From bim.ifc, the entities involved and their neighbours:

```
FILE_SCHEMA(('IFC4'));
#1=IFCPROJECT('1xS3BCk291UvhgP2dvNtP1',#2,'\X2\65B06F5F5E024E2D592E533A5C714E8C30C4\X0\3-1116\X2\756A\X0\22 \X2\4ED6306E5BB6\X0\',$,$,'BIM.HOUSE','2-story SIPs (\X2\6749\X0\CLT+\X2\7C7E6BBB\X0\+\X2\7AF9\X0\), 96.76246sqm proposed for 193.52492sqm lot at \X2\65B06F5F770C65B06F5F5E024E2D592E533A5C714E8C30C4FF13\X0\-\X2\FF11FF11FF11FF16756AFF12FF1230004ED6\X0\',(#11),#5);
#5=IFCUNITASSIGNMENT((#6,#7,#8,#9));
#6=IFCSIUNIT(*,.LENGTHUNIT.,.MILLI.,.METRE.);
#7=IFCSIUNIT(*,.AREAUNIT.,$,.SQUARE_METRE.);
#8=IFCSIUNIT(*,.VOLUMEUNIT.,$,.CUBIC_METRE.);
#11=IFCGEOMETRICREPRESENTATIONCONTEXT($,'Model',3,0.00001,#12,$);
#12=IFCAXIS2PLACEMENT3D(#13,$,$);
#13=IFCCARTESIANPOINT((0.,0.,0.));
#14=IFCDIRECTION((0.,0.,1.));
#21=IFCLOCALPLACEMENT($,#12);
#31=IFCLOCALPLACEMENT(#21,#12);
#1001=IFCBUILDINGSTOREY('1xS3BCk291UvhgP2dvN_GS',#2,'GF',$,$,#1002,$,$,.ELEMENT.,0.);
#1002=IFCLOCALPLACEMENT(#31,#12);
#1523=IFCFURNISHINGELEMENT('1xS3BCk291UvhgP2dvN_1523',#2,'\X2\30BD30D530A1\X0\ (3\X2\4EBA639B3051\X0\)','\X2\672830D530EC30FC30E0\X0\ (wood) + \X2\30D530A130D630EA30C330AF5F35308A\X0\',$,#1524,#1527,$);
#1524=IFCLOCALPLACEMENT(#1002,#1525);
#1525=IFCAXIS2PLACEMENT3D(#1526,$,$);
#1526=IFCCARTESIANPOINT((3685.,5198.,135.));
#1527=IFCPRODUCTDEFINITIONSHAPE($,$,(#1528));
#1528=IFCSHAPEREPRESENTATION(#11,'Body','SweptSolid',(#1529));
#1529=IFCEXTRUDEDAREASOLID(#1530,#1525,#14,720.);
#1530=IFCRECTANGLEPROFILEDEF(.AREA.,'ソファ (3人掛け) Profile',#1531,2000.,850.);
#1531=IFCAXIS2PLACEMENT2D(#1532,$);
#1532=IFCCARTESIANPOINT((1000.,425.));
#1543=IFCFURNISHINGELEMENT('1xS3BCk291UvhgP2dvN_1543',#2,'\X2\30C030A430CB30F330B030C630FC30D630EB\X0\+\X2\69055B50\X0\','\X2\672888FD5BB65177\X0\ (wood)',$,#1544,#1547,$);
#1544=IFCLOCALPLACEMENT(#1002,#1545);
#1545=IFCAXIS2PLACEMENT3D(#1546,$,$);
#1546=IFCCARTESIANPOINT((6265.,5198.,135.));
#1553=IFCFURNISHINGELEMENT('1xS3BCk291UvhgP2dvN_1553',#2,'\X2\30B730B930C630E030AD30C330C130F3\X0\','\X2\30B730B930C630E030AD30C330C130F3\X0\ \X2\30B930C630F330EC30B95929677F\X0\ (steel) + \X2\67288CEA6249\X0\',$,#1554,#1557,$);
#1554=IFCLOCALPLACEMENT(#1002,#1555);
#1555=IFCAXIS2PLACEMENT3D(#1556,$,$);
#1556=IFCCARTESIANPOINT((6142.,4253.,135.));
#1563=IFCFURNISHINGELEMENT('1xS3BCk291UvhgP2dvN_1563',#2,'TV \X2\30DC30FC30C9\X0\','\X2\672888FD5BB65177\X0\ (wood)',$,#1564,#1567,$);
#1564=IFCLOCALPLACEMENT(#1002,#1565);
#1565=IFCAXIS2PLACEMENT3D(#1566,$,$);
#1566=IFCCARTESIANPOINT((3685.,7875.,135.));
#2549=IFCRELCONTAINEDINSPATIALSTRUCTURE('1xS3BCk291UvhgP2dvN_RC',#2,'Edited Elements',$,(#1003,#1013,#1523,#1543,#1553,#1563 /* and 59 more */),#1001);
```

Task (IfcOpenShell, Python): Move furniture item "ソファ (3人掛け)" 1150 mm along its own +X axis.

```python
import ifcopenshell
import ifcopenshell.api.geometry
import ifcopenshell.util.placement

model = ifcopenshell.open("bim.ifc")

item = model.by_guid("1xS3BCk291UvhgP2dvN_1523")
matrix = ifcopenshell.util.placement.get_local_placement(item.ObjectPlacement)
matrix[:3, 3] += matrix[:3, 0] * 1150.0
ifcopenshell.api.geometry.edit_object_placement(model, product=item, matrix=matrix, is_si=False)

print(ifcopenshell.util.placement.get_local_placement(item.ObjectPlacement).round(3) + 0.0)

model.write("bim_updated.ifc")
```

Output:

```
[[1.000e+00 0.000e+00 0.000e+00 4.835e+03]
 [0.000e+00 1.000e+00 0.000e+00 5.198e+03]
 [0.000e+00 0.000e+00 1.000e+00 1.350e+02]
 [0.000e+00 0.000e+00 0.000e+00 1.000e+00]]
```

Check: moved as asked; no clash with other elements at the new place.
